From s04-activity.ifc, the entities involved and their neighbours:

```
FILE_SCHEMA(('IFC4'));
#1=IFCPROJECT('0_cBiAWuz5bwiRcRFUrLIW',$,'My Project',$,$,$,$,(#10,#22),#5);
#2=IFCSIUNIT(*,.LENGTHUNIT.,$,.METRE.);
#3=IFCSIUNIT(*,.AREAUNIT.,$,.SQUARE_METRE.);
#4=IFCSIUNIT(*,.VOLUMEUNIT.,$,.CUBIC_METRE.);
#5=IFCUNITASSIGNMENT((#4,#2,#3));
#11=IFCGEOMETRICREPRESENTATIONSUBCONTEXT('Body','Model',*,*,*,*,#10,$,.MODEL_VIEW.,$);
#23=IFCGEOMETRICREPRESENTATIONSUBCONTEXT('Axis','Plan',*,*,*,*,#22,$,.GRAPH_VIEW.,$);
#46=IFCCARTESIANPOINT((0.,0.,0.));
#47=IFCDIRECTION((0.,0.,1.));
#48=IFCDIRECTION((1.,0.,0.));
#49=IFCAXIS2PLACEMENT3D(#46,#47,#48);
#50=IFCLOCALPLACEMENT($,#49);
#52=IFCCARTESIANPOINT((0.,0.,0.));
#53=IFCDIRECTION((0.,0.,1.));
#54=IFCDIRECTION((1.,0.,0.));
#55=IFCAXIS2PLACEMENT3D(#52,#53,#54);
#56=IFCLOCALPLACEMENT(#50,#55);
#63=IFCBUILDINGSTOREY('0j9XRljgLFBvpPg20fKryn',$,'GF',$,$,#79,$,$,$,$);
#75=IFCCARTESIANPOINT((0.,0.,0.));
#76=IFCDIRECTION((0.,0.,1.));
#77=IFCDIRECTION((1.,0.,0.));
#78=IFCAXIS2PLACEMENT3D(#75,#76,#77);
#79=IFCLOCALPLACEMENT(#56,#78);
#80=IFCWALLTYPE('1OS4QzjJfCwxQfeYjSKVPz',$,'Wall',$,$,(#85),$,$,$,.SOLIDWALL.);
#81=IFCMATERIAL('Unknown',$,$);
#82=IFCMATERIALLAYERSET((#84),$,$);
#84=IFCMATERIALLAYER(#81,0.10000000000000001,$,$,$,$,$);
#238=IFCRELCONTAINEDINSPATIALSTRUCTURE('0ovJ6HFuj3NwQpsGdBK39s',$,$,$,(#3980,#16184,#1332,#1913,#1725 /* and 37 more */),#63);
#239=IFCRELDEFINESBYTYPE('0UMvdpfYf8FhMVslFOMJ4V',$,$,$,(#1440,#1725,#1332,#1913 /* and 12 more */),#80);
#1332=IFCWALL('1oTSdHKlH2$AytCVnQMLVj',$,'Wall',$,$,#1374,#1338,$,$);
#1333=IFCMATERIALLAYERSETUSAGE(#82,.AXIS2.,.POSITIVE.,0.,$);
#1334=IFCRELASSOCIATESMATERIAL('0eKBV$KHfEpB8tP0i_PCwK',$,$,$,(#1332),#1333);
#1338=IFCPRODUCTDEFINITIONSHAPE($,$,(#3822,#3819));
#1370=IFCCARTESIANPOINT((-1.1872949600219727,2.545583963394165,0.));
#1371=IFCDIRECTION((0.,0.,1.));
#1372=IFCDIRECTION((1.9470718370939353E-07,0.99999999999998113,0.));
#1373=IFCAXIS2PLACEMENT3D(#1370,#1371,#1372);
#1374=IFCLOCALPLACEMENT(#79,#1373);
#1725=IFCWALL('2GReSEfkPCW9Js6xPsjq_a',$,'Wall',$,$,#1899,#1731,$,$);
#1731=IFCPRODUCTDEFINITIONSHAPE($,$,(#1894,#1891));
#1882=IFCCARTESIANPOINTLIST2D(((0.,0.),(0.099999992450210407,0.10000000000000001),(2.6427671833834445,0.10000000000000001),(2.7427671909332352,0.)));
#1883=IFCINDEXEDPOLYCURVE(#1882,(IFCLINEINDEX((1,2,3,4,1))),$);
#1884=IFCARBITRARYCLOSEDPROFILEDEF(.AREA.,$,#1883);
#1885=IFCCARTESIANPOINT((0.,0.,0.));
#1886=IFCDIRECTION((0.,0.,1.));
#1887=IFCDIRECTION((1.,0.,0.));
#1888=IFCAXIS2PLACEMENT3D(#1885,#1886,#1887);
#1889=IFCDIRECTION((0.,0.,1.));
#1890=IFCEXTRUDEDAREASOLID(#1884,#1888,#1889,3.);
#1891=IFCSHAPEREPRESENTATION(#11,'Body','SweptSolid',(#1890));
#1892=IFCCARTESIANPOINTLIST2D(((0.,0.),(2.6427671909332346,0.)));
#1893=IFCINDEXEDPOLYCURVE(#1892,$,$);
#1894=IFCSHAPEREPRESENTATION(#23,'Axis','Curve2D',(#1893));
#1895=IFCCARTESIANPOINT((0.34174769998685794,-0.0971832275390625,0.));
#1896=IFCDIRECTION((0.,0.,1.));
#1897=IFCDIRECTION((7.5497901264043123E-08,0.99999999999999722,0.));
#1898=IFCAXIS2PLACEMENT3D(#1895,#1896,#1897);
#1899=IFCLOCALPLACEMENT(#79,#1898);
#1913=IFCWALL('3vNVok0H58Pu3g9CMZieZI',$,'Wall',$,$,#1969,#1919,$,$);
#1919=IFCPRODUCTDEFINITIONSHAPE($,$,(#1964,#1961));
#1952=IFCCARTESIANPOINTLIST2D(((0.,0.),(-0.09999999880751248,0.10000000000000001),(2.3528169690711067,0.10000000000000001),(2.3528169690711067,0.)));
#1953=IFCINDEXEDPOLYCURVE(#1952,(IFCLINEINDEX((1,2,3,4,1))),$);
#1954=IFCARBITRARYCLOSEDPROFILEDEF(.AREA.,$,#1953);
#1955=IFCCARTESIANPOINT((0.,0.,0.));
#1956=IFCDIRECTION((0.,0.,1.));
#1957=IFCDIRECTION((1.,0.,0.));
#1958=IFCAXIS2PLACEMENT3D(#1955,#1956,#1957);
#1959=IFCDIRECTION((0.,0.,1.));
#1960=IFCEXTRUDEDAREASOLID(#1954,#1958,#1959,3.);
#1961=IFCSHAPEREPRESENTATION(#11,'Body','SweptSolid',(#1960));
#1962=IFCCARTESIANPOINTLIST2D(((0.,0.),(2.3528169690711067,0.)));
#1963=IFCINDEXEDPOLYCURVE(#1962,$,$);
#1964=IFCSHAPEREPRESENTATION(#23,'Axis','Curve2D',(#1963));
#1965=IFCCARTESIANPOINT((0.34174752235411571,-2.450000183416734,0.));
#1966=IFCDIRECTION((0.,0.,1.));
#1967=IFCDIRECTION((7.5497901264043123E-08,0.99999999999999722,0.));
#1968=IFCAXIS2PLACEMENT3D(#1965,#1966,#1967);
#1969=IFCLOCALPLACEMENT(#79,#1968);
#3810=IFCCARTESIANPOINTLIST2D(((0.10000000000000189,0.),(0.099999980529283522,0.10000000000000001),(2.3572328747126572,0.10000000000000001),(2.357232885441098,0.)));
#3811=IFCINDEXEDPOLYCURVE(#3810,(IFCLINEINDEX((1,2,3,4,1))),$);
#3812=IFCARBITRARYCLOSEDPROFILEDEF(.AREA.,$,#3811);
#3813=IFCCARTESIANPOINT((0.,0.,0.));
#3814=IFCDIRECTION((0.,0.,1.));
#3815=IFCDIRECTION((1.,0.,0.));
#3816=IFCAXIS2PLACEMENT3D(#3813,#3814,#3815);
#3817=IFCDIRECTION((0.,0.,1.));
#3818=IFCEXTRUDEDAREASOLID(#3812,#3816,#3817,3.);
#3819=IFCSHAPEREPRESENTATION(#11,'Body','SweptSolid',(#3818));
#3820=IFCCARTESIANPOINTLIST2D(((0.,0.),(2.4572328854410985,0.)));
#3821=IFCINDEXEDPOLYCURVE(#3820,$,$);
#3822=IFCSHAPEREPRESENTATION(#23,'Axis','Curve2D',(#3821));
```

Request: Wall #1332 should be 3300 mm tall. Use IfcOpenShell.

```python
import ifcopenshell
import ifcopenshell.geom
import ifcopenshell.util.representation
import ifcopenshell.util.shape
import ifcopenshell.util.unit

model = ifcopenshell.open("s04-activity.ifc")
unit_scale = ifcopenshell.util.unit.calculate_unit_scale(model)
settings = ifcopenshell.geom.settings()


def volume(element):
    """Net volume in cubic metres, openings subtracted."""
    shape = ifcopenshell.geom.create_shape(settings, element)
    return ifcopenshell.util.shape.get_volume(shape.geometry)


wall = model.by_guid("1oTSdHKlH2$AytCVnQMLVj")
before = volume(wall)

body = ifcopenshell.util.representation.get_representation(wall, "Model", "Body")
solid = body.Items[0]
old_height = solid.Depth
solid.Depth = 3.3 / unit_scale
after = volume(wall)

print(f"height {old_height:g} -> {solid.Depth:g}, volume {before:.3f} -> {after:.3f} m3")

model.write("s04-activity_edited.ifc")
```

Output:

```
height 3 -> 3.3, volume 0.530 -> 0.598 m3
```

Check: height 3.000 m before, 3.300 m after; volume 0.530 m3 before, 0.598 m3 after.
